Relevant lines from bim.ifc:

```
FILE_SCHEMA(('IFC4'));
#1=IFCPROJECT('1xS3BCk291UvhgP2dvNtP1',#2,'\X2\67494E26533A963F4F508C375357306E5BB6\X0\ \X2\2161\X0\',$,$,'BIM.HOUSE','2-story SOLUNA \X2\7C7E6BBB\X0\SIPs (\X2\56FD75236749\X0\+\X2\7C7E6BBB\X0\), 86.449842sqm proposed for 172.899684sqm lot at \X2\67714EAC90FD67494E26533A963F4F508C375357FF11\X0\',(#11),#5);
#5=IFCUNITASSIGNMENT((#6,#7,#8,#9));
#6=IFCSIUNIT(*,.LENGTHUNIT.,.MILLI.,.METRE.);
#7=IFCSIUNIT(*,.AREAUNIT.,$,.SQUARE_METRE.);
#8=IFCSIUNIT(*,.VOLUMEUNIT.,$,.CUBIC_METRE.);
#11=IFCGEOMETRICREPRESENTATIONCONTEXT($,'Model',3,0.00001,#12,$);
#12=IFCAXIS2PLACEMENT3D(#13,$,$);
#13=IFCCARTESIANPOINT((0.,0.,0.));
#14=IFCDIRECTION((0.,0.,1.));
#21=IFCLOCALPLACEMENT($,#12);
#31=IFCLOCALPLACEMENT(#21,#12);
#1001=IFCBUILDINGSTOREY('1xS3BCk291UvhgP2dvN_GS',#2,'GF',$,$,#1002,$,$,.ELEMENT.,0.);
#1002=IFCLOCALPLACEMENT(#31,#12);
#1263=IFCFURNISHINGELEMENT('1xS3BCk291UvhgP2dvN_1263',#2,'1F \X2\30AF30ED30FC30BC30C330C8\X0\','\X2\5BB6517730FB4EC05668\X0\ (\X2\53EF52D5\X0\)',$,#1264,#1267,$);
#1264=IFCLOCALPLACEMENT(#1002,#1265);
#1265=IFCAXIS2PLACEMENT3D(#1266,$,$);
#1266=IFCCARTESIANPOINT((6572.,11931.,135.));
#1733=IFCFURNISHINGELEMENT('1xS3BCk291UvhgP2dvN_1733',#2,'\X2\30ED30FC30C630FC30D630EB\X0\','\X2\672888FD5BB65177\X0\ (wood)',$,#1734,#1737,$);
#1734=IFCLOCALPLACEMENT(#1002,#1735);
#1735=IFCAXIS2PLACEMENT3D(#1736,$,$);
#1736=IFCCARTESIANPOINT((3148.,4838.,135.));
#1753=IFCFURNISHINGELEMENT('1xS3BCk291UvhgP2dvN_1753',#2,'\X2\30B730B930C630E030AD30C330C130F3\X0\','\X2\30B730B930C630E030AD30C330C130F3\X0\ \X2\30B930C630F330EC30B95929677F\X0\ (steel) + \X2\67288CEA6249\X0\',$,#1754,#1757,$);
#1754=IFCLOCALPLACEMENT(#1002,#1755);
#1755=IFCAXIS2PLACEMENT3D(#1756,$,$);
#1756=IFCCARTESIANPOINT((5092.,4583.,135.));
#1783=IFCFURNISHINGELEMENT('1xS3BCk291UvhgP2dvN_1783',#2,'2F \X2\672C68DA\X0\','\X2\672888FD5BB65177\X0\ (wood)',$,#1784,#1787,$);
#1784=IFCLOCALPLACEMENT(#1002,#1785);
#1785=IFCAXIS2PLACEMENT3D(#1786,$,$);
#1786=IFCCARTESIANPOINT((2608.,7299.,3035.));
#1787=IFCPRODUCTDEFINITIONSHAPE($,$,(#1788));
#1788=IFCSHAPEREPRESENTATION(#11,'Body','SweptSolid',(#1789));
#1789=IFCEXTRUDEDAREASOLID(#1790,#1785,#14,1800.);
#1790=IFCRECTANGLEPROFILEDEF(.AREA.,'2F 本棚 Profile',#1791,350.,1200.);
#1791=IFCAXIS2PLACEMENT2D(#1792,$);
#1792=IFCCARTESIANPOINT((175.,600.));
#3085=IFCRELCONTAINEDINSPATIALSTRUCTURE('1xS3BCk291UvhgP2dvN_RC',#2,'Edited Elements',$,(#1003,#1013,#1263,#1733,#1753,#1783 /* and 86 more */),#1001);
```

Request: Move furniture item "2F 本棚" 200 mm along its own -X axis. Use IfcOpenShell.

```python
import ifcopenshell
import ifcopenshell.api.geometry
import ifcopenshell.util.placement
import ifcopenshell.util.unit

model = ifcopenshell.open("bim.ifc")
unit_scale = ifcopenshell.util.unit.calculate_unit_scale(model)

item = model.by_guid("1xS3BCk291UvhgP2dvN_1783")
matrix = ifcopenshell.util.placement.get_local_placement(item.ObjectPlacement)
matrix[:3, 3] -= matrix[:3, 0] * 0.2 / unit_scale
ifcopenshell.api.geometry.edit_object_placement(model, product=item, matrix=matrix, is_si=False)

print(ifcopenshell.util.placement.get_local_placement(item.ObjectPlacement).round(3) + 0.0)

model.write("bim_rev.ifc")
```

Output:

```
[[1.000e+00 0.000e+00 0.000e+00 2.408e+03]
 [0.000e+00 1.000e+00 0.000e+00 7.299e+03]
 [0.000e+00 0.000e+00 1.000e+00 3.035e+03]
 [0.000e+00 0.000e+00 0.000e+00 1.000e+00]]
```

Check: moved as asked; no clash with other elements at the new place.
